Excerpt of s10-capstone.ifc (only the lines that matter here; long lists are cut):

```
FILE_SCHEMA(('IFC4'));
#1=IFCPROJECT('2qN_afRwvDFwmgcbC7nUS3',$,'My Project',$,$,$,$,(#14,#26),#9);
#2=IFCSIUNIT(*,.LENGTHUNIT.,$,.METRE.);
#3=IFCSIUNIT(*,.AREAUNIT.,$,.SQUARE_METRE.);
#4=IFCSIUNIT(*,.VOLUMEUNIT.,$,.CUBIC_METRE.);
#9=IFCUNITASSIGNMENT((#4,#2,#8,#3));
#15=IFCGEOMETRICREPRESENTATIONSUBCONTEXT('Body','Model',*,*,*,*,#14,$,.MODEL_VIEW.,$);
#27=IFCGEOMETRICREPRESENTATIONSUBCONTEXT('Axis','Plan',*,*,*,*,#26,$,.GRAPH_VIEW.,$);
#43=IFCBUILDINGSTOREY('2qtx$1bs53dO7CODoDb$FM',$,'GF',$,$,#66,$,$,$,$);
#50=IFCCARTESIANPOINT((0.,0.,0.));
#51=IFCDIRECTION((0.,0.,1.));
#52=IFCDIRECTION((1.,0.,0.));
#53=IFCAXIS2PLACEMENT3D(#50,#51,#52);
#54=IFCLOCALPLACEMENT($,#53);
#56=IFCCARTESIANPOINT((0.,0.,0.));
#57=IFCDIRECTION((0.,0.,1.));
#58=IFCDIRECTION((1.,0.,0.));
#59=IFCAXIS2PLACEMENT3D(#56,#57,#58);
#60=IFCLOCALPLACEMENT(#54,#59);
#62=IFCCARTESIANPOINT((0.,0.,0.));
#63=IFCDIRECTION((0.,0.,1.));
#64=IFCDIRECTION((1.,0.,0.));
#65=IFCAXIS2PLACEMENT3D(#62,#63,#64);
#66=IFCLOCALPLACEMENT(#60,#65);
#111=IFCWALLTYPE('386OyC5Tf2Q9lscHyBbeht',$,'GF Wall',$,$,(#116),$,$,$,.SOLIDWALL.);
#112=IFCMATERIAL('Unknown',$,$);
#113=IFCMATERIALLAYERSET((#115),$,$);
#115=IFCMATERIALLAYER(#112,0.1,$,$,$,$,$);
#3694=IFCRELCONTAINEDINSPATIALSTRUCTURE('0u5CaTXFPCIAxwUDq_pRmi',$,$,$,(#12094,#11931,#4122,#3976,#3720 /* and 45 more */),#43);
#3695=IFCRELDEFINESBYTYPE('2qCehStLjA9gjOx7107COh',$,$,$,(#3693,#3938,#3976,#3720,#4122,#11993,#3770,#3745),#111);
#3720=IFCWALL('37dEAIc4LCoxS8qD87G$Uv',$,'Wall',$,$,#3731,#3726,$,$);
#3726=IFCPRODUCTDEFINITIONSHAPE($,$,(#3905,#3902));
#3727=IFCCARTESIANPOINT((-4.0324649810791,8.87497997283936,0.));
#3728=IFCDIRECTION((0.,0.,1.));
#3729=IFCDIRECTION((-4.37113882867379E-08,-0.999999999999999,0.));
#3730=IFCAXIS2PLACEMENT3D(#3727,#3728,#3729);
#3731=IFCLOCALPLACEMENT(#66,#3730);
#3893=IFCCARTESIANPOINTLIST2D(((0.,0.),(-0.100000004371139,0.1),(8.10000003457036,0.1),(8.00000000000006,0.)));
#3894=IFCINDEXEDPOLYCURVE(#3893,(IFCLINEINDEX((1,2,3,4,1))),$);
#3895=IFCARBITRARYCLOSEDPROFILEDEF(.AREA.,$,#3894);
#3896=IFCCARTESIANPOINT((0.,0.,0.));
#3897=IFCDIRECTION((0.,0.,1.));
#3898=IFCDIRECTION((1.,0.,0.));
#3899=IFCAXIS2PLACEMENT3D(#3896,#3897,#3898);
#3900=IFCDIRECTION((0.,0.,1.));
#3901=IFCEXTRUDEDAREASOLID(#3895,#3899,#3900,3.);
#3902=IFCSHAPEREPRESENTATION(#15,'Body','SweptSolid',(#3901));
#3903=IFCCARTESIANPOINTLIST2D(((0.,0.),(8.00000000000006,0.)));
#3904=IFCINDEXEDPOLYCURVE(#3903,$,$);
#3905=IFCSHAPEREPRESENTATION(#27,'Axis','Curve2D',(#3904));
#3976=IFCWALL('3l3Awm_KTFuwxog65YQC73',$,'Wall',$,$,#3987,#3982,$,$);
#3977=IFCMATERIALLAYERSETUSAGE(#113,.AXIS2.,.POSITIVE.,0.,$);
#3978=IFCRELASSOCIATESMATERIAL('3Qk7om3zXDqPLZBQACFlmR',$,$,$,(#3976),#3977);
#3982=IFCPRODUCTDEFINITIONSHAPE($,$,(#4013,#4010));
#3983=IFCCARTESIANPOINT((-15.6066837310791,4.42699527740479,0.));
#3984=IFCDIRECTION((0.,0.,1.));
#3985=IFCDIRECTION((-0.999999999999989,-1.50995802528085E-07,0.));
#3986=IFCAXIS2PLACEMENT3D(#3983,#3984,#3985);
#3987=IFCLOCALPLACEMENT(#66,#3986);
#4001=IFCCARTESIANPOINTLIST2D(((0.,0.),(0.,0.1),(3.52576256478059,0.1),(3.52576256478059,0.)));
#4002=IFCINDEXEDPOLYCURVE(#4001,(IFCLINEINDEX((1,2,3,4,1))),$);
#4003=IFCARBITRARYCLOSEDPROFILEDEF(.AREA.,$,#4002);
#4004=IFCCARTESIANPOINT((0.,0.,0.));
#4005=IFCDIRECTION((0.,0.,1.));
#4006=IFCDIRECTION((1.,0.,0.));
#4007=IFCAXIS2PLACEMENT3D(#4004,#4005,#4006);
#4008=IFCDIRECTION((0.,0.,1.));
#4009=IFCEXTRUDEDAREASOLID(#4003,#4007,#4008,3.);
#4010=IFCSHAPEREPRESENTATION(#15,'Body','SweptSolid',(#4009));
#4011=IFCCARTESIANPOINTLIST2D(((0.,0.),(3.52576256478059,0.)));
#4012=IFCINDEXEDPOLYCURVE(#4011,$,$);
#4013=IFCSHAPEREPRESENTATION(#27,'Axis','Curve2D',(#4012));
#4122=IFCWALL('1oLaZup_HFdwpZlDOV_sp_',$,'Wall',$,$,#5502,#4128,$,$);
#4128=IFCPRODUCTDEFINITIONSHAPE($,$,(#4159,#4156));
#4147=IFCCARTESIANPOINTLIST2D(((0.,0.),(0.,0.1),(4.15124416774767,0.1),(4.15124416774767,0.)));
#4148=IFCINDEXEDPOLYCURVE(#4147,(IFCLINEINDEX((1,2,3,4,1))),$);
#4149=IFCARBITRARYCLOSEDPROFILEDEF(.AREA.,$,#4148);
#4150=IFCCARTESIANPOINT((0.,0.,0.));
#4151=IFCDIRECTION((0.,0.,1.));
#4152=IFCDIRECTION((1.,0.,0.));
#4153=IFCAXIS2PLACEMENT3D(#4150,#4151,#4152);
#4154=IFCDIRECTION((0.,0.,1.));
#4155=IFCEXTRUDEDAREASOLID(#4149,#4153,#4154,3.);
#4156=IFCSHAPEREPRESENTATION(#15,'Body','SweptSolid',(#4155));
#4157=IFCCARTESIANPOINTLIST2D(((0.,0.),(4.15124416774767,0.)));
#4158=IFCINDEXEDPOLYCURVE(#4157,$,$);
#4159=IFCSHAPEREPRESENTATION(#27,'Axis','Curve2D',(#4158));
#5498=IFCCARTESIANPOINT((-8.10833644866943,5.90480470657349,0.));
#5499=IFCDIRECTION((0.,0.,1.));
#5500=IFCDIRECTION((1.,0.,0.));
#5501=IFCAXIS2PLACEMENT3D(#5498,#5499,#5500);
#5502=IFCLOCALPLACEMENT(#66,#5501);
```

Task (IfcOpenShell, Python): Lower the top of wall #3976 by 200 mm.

```python
import ifcopenshell
import ifcopenshell.geom
import ifcopenshell.util.representation
import ifcopenshell.util.shape

model = ifcopenshell.open("s10-capstone.ifc")
settings = ifcopenshell.geom.settings()


def volume(element):
    """Net volume in cubic metres, openings subtracted."""
    shape = ifcopenshell.geom.create_shape(settings, element)
    return ifcopenshell.util.shape.get_volume(shape.geometry)


wall = model.by_guid("3l3Awm_KTFuwxog65YQC73")
before = volume(wall)

body = ifcopenshell.util.representation.get_representation(wall, "Model", "Body")
solid = body.Items[0]
old_height = solid.Depth
solid.Depth -= 0.2
after = volume(wall)

print(f"height {old_height:g} -> {solid.Depth:g}, volume {before:.3f} -> {after:.3f} m3")

model.write("s10-capstone_v2.ifc")
```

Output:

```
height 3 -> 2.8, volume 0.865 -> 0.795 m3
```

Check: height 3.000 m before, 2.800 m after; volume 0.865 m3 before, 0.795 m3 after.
